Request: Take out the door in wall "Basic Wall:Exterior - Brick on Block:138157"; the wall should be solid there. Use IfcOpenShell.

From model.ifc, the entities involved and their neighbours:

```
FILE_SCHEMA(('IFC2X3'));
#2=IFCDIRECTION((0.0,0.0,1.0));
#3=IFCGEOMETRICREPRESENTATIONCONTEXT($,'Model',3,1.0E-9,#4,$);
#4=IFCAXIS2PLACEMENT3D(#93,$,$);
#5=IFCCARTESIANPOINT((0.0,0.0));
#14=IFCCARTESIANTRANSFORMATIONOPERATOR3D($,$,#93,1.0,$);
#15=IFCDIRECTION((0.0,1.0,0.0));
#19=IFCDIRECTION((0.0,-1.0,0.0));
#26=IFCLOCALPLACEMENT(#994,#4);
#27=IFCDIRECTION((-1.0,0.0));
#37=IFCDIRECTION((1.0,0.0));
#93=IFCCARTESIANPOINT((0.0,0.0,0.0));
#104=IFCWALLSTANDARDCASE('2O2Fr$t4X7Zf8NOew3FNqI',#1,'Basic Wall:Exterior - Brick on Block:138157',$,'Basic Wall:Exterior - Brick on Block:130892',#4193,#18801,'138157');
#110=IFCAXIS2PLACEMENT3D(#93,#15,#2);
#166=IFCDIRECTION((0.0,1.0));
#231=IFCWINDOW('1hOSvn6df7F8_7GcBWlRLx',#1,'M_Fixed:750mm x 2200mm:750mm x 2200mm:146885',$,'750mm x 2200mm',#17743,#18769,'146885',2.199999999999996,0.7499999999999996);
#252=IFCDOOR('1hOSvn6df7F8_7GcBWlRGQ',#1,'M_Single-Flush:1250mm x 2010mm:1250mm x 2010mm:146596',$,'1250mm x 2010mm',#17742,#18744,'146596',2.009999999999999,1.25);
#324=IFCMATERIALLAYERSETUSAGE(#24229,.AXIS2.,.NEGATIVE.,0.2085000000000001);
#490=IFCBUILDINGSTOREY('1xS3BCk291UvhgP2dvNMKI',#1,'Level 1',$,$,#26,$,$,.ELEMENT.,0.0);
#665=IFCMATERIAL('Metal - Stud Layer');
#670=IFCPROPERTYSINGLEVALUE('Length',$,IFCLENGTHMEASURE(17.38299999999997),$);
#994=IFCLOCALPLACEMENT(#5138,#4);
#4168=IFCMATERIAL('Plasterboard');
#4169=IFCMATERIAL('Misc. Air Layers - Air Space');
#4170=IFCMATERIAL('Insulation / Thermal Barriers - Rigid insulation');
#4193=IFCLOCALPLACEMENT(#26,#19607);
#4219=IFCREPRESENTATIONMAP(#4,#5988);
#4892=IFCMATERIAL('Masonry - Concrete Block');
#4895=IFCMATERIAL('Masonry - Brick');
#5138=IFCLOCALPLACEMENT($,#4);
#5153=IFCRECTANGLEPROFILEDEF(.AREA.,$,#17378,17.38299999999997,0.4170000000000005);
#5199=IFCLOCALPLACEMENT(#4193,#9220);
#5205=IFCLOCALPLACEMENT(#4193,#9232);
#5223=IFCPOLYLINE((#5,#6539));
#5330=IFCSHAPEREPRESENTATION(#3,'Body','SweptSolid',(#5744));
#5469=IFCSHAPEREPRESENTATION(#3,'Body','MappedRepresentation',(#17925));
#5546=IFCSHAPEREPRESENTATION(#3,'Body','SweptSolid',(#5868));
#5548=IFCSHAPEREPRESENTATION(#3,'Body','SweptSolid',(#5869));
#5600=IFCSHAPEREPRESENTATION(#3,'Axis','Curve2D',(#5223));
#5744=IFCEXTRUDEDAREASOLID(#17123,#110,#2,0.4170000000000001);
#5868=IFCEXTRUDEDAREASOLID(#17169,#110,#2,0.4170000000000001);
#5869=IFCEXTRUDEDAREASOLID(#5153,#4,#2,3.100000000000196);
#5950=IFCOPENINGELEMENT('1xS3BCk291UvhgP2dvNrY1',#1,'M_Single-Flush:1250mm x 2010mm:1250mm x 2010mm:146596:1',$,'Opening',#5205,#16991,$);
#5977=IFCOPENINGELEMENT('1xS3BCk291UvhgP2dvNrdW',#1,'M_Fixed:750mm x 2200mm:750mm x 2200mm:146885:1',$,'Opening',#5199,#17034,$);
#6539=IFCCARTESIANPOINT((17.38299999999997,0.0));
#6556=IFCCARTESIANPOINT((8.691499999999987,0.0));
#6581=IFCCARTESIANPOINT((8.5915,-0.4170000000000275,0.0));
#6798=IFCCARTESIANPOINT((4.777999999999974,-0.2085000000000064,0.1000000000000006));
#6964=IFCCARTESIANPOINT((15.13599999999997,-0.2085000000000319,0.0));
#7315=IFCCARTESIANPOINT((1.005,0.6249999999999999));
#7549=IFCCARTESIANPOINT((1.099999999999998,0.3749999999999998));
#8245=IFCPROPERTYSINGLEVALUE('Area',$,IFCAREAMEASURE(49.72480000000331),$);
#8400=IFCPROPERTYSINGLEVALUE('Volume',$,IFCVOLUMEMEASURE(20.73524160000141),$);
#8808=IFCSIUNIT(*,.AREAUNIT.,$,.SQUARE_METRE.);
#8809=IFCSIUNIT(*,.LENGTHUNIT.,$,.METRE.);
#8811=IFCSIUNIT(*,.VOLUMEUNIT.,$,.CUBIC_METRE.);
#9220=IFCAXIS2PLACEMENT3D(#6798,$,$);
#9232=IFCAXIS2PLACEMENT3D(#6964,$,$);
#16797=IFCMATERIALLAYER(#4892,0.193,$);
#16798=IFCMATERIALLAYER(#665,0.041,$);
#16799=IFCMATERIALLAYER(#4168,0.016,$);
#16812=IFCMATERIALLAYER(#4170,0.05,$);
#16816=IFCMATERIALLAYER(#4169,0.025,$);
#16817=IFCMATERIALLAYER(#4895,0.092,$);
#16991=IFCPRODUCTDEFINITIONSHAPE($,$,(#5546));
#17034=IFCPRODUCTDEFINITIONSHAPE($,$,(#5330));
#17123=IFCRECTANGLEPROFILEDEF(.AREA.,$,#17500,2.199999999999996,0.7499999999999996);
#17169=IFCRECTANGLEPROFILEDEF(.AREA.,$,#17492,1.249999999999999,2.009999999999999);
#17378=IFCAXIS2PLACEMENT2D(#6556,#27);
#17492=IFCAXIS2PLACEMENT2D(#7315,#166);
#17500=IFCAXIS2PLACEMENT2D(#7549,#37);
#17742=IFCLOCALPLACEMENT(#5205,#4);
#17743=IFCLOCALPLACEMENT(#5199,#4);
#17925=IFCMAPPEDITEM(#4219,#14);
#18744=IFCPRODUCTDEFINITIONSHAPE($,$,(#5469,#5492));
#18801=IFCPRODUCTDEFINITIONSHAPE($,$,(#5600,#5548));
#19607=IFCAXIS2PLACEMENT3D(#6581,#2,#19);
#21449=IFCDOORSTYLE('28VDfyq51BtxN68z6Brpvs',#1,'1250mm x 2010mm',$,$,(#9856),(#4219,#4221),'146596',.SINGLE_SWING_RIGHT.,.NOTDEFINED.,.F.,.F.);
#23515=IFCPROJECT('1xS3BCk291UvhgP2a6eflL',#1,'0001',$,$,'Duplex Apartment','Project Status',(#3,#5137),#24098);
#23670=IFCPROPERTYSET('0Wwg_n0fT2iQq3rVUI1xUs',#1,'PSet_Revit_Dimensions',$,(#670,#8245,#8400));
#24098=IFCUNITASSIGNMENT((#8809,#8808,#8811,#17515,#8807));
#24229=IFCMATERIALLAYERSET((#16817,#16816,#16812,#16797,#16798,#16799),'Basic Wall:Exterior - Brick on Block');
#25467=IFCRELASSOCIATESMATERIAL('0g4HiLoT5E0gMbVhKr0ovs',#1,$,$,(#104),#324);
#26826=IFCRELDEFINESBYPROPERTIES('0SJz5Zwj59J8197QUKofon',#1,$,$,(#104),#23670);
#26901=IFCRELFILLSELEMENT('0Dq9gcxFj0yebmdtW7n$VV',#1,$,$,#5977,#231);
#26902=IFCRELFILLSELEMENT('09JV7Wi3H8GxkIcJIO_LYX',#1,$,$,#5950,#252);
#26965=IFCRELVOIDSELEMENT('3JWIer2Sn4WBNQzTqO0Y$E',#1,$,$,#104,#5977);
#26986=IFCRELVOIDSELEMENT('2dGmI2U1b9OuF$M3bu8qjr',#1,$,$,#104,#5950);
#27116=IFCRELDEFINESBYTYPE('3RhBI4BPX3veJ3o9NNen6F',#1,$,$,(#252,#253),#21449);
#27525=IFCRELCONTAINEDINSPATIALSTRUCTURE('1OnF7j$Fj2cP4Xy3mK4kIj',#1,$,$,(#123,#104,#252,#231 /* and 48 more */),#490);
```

```python
import ifcopenshell
import ifcopenshell.api.feature
import ifcopenshell.api.pset
import ifcopenshell.api.root
import ifcopenshell.geom
import ifcopenshell.util.element
import ifcopenshell.util.shape
import ifcopenshell.util.unit

model = ifcopenshell.open("model.ifc")
area_scale = ifcopenshell.util.unit.calculate_unit_scale(model, "AREAUNIT")
volume_scale = ifcopenshell.util.unit.calculate_unit_scale(model, "VOLUMEUNIT")
settings = ifcopenshell.geom.settings()


def volume(element):
    """Net volume in cubic metres, openings subtracted."""
    shape = ifcopenshell.geom.create_shape(settings, element)
    return ifcopenshell.util.shape.get_volume(shape.geometry)


door = model.by_guid("1hOSvn6df7F8_7GcBWlRGQ")
opening = door.FillsVoids[0].RelatingOpeningElement
wall = opening.VoidsElements[0].RelatingBuildingElement
before = volume(wall)

ifcopenshell.api.root.remove_product(model, product=door)
ifcopenshell.api.feature.remove_feature(model, feature=opening)

after = volume(wall)
thickness = 0.417  # wall thickness in metres

# Update the wall's stored quantities.
pset = model.by_id(ifcopenshell.util.element.get_pset(wall, "PSet_Revit_Dimensions", should_inherit=False)["id"])
ifcopenshell.api.pset.edit_pset(model, pset=pset, properties={
    "Area": model.create_entity("IfcAreaMeasure", after / thickness / area_scale),
    "Volume": model.create_entity("IfcVolumeMeasure", after / volume_scale),
})

print(f"wall volume {before:.3f} -> {after:.3f} m3")

model.write("model_edited.ifc")
```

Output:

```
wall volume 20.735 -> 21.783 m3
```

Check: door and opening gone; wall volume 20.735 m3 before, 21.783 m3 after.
